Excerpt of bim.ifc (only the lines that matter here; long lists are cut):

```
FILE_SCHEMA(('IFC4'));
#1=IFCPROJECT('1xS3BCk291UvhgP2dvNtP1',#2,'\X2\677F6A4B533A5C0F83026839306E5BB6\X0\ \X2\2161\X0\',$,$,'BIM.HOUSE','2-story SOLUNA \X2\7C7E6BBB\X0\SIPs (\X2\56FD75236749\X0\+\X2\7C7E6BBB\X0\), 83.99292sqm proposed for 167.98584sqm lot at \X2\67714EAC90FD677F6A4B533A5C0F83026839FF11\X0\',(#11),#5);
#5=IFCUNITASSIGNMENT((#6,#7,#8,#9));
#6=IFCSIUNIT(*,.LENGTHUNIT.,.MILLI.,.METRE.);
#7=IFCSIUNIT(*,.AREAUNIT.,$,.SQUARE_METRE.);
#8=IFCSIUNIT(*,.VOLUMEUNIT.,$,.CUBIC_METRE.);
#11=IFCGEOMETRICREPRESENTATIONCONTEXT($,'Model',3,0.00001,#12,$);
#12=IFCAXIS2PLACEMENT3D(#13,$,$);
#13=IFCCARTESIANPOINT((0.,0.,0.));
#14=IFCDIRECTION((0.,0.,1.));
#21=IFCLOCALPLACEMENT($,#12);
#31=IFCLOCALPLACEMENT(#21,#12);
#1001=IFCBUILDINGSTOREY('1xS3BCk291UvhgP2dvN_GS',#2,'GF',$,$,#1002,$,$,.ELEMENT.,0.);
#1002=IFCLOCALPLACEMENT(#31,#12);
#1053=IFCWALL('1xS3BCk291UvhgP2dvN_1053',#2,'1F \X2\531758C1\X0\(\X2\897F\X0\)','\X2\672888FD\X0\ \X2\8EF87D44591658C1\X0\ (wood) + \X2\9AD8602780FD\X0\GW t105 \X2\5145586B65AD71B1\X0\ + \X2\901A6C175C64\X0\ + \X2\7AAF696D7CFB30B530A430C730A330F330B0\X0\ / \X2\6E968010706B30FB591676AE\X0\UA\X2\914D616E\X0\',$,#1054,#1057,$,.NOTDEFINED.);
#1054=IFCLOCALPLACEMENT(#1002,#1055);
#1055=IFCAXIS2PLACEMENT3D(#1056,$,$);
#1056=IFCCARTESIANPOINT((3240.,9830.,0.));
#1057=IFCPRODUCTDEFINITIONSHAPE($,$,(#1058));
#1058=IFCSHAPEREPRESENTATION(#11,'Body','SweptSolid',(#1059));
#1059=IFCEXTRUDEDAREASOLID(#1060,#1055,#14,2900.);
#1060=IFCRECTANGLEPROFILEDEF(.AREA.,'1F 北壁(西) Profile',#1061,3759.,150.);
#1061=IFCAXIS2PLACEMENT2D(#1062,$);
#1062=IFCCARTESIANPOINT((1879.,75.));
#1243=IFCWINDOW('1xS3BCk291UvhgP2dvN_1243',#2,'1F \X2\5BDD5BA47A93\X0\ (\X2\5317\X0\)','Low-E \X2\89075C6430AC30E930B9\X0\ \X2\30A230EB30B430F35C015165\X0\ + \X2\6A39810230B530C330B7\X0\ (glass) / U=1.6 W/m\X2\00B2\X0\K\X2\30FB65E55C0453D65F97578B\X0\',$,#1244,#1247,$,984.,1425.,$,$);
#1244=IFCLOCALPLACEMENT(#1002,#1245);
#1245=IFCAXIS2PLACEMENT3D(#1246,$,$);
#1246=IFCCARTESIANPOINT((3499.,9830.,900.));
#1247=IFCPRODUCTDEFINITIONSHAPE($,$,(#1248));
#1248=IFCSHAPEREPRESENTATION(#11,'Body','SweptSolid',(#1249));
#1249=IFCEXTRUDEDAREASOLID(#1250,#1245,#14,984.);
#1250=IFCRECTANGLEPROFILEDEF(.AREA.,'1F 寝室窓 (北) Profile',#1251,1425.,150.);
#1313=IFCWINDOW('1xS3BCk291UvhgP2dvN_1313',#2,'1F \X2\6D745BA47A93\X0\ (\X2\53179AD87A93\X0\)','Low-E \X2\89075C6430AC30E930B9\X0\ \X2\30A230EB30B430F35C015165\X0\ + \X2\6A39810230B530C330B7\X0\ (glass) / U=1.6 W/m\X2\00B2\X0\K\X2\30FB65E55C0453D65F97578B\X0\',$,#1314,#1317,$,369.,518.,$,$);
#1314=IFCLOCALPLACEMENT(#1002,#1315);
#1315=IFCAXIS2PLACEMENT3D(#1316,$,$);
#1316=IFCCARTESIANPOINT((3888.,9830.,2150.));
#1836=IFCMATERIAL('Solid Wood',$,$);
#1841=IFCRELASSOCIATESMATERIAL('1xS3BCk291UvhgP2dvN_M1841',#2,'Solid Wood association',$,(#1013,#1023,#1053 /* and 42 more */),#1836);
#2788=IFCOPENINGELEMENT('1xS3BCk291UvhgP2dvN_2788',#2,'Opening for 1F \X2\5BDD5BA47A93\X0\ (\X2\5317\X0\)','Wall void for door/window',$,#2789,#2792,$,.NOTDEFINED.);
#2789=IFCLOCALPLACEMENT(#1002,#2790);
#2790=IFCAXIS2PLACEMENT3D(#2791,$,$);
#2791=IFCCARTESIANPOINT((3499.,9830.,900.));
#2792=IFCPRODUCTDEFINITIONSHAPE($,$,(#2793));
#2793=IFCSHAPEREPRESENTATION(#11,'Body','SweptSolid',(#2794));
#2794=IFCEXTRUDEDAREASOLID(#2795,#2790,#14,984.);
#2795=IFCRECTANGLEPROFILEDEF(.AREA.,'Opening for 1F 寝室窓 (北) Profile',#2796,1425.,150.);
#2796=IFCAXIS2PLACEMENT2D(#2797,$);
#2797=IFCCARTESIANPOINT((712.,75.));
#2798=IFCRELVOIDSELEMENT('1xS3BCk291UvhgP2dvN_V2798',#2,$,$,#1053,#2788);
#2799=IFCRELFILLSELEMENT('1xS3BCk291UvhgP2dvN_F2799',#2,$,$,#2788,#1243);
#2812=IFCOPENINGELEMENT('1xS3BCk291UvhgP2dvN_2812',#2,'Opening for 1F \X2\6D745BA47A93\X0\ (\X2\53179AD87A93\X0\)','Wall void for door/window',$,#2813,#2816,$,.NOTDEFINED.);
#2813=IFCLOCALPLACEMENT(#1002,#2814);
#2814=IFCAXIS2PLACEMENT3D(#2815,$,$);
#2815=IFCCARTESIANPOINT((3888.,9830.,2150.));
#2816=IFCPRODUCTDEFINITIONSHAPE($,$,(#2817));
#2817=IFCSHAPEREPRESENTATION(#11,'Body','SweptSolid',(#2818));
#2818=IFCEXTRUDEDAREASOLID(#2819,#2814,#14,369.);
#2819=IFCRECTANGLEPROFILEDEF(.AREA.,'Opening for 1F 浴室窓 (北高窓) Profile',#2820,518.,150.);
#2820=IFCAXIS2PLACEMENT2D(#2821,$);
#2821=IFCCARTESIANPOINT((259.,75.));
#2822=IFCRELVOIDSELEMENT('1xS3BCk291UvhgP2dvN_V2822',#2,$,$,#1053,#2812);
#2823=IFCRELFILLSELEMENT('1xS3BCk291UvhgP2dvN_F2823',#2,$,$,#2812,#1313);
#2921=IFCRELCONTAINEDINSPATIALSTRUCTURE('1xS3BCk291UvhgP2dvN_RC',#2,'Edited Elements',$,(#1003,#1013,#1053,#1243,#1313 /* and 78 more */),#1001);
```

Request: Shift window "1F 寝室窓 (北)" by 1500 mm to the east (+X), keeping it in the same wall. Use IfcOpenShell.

```python
import ifcopenshell
import ifcopenshell.api.geometry
import ifcopenshell.util.placement

model = ifcopenshell.open("bim.ifc")

window = model.by_guid("1xS3BCk291UvhgP2dvN_1243")
opening = window.FillsVoids[0].RelatingOpeningElement
wall = opening.VoidsElements[0].RelatingBuildingElement

wall_matrix = ifcopenshell.util.placement.get_local_placement(wall.ObjectPlacement)
shift = wall_matrix[:3, 0] * 1500.0
before = ifcopenshell.util.placement.get_local_placement(window.ObjectPlacement)[:3, 3].copy()

# The window is not placed relative to its opening, so move both.
for product in (opening, window):
    matrix = ifcopenshell.util.placement.get_local_placement(product.ObjectPlacement)
    matrix[:3, 3] += shift
    ifcopenshell.api.geometry.edit_object_placement(model, product=product, matrix=matrix, is_si=False)

after = ifcopenshell.util.placement.get_local_placement(window.ObjectPlacement)[:3, 3]
print("window moved by", (after - before).round(3) + 0.0)

model.write("bim-out.ifc")
```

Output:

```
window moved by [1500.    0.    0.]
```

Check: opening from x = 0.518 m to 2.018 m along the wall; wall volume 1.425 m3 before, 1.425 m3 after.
